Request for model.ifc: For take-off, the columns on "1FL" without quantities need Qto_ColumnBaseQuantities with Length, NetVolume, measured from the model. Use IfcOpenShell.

First a look at what the model holds.

```python
import ifcopenshell
import ifcopenshell.util.element
import ifcopenshell.util.unit

model = ifcopenshell.open("model.ifc")
print(model.schema)
for unit_type in ("LENGTHUNIT", "AREAUNIT", "VOLUMEUNIT"):
    print(unit_type, ifcopenshell.util.unit.calculate_unit_scale(model, unit_type))
storey = next(s for s in model.by_type("IfcBuildingStorey") if s.Name == "1FL")
columns = [e for e in ifcopenshell.util.element.get_decomposition(storey) if e.is_a("IfcColumn")]
for e in sorted(columns, key=lambda e: e.id()):
    print(e.id(), e.is_a(), e.Name, list(ifcopenshell.util.element.get_psets(e, qtos_only=True)), sep=" | ")
```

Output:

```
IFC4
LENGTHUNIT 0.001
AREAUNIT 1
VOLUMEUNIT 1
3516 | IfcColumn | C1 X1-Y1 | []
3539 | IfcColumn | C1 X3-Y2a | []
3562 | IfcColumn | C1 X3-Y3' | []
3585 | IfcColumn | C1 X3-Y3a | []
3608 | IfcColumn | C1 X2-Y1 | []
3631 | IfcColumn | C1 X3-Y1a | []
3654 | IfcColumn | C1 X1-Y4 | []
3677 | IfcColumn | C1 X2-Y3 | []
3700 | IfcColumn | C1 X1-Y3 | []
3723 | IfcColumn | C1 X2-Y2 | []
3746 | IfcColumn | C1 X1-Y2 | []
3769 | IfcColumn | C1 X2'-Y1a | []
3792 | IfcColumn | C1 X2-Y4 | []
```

```python
import ifcopenshell
import ifcopenshell.api.pset
import ifcopenshell.geom
import ifcopenshell.util.element
import ifcopenshell.util.shape
import ifcopenshell.util.unit

model = ifcopenshell.open("model.ifc")
unit_scale = ifcopenshell.util.unit.calculate_unit_scale(model)
volume_scale = ifcopenshell.util.unit.calculate_unit_scale(model, "VOLUMEUNIT")
settings = ifcopenshell.geom.settings()

storey = next(s for s in model.by_type("IfcBuildingStorey") if s.Name == "1FL")
columns = [e for e in ifcopenshell.util.element.get_decomposition(storey) if e.is_a("IfcColumn")]

for e in sorted(columns, key=lambda e: e.id()):
    if ifcopenshell.util.element.get_psets(e, qtos_only=True, should_inherit=False):
        continue
    # Geometry comes back in metres, in the element's own axes.
    shape = ifcopenshell.geom.create_shape(settings, e)
    values = {
        "Length": ifcopenshell.util.shape.get_z(shape.geometry) / unit_scale,
        "NetVolume": ifcopenshell.util.shape.get_volume(shape.geometry) / volume_scale,
    }
    qto = ifcopenshell.api.pset.add_qto(model, product=e, name="Qto_ColumnBaseQuantities")
    ifcopenshell.api.pset.edit_qto(model, qto=qto, properties=values)
    print(e.id(), {k: round(v, 3) for k, v in values.items()})

model.write("model-out.ifc")
```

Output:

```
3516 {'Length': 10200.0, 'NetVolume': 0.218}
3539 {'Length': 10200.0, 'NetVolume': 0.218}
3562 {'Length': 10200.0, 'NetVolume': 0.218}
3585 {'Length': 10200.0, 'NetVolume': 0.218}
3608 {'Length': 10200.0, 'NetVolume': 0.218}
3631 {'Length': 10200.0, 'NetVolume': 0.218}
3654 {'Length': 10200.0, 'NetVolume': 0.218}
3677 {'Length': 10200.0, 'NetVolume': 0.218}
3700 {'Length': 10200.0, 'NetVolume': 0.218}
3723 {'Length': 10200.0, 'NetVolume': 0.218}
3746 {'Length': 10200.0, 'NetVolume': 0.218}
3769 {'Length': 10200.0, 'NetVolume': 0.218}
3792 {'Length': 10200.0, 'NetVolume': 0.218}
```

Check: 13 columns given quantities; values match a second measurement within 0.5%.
